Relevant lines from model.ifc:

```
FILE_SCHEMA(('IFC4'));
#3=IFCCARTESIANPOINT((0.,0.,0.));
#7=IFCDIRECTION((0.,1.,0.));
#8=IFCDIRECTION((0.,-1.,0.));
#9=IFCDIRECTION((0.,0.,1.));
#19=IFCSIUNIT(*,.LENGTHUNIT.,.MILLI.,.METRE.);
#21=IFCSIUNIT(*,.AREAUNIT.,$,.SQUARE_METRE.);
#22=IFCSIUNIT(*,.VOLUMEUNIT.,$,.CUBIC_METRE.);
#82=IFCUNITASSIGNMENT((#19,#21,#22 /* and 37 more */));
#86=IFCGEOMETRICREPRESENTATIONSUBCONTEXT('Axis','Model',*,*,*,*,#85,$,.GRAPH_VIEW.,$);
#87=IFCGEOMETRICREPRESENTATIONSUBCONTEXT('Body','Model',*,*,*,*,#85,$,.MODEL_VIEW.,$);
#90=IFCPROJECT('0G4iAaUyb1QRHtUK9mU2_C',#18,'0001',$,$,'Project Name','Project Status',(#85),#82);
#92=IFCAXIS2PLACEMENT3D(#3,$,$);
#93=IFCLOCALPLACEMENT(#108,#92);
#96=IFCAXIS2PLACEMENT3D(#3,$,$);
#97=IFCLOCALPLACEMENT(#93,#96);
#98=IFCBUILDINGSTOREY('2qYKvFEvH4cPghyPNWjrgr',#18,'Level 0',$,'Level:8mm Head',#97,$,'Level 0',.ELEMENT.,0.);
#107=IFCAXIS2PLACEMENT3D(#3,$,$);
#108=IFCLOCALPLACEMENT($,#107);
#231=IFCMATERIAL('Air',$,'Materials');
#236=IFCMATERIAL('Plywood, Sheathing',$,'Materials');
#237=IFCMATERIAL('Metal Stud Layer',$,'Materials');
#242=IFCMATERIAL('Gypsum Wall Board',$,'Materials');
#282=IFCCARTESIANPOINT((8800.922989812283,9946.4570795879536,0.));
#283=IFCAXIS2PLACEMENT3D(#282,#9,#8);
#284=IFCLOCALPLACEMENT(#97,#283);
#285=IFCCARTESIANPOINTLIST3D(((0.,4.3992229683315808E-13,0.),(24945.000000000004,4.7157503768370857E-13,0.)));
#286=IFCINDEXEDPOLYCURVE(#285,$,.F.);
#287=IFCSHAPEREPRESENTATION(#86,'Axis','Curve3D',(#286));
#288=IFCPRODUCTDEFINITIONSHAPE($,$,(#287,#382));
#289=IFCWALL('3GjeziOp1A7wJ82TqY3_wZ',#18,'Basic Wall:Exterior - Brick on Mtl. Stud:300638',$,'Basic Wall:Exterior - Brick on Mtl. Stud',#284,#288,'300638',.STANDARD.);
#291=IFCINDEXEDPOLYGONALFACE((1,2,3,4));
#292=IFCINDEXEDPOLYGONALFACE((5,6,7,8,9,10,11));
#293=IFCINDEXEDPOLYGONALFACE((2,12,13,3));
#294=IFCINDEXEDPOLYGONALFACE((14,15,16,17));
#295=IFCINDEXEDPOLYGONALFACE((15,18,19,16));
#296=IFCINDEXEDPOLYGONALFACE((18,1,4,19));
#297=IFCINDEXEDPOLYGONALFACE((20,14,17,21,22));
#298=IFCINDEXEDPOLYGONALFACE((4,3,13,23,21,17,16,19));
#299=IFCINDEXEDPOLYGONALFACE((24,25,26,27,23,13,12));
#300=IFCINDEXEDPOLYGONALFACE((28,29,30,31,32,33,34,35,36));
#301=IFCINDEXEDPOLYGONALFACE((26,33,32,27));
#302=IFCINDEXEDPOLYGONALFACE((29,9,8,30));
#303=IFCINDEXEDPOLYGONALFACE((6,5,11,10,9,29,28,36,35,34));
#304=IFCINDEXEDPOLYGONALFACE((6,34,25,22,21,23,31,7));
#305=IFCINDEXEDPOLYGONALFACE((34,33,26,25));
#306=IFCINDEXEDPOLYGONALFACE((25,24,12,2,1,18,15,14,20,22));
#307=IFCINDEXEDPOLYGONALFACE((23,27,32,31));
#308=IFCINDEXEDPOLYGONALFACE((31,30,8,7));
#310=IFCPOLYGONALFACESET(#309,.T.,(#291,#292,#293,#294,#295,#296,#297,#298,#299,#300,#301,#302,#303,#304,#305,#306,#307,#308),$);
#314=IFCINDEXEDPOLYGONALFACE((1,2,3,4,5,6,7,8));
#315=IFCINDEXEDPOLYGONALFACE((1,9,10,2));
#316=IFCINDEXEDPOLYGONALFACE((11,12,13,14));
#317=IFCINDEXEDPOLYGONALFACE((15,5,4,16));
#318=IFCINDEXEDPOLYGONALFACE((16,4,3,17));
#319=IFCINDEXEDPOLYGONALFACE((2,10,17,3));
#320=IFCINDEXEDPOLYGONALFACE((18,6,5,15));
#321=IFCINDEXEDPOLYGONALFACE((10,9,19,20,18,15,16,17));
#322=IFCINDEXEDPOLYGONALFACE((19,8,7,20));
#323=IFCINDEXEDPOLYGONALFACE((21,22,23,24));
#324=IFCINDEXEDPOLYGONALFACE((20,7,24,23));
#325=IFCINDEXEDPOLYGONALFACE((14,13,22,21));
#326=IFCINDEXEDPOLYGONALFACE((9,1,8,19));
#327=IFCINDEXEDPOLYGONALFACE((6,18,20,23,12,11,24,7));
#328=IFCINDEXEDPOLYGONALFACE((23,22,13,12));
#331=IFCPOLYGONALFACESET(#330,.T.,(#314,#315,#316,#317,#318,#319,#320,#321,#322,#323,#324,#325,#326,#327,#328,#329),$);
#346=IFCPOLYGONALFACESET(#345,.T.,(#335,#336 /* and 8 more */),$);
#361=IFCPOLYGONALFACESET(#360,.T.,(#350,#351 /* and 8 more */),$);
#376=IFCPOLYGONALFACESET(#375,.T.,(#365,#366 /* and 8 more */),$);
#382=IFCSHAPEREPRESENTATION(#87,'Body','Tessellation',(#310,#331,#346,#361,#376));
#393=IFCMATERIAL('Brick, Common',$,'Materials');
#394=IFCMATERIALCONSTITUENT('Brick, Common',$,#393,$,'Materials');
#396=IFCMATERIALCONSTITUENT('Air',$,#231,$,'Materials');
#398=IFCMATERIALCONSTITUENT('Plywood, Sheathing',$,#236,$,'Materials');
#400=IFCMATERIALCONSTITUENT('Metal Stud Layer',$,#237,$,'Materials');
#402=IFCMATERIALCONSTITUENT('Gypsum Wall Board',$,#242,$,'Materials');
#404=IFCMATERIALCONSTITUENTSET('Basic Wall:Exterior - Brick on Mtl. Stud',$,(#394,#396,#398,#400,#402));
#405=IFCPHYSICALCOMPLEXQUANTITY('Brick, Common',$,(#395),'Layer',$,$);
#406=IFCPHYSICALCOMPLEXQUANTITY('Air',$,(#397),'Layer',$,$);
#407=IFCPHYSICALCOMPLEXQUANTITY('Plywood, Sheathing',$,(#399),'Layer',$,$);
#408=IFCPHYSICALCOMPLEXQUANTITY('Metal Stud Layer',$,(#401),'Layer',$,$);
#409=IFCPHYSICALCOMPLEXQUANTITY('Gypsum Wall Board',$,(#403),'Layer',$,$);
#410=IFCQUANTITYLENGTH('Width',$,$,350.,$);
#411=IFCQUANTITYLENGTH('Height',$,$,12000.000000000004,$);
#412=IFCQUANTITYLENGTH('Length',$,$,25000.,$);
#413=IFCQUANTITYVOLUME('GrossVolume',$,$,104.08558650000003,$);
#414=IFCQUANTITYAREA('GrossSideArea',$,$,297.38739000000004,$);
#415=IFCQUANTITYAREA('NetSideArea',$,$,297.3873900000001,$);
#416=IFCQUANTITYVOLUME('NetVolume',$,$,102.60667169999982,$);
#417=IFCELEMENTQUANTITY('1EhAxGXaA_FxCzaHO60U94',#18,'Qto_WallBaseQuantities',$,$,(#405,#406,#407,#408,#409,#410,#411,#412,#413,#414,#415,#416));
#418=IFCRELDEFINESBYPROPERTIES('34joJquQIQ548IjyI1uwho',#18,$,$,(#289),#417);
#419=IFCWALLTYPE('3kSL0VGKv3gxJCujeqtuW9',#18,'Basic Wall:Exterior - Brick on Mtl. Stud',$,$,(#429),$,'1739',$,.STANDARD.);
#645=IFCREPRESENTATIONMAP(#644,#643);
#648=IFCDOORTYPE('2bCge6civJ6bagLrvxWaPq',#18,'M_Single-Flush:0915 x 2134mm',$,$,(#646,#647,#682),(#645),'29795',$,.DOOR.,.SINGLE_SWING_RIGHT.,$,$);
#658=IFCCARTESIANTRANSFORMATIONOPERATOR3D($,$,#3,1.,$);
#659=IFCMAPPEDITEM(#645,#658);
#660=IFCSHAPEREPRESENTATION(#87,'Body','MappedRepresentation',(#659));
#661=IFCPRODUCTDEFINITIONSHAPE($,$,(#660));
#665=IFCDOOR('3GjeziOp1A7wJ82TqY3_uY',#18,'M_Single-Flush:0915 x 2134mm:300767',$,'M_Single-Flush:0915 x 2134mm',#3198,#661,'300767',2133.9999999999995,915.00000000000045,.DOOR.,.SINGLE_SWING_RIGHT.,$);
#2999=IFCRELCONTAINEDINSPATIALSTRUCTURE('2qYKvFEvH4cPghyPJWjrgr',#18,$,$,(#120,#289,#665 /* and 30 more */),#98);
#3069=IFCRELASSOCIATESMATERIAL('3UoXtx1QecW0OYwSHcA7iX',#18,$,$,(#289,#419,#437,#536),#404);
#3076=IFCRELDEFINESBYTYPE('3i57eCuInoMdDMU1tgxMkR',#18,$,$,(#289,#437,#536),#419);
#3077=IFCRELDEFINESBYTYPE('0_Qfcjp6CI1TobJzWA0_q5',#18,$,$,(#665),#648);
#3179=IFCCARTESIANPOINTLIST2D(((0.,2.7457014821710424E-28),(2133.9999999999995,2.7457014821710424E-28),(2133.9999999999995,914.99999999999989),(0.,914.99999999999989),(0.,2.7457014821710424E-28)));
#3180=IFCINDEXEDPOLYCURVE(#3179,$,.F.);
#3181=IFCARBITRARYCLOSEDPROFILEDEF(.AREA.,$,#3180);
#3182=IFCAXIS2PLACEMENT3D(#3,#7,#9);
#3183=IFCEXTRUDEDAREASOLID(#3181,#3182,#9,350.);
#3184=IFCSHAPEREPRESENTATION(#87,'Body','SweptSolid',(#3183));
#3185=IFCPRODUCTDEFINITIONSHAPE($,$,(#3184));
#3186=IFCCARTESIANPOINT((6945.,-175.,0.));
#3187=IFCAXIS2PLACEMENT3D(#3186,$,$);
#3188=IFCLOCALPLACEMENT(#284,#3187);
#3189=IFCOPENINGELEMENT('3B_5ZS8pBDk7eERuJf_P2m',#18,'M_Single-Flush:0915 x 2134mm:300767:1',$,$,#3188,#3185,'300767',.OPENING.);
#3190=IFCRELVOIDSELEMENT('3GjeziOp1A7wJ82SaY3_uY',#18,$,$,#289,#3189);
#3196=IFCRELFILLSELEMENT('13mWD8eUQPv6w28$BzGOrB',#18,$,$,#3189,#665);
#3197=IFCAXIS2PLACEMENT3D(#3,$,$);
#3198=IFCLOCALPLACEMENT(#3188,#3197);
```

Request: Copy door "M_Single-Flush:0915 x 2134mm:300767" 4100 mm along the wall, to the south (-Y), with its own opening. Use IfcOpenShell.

```python
import ifcopenshell
import ifcopenshell.api.feature
import ifcopenshell.api.geometry
import ifcopenshell.api.pset
import ifcopenshell.api.root
import ifcopenshell.geom
import ifcopenshell.util.element
import ifcopenshell.util.placement
import ifcopenshell.util.shape
import ifcopenshell.util.unit

model = ifcopenshell.open("model.ifc")
area_scale = ifcopenshell.util.unit.calculate_unit_scale(model, "AREAUNIT")
volume_scale = ifcopenshell.util.unit.calculate_unit_scale(model, "VOLUMEUNIT")
settings = ifcopenshell.geom.settings()


def volume(element):
    """Net volume in cubic metres, openings subtracted."""
    shape = ifcopenshell.geom.create_shape(settings, element)
    return ifcopenshell.util.shape.get_volume(shape.geometry)


def reuse_history(source, copy):
    """copy_class also copies each property set's owner history, people and application; keep the originals."""
    for rel in copy.IsDefinedBy:
        if rel.is_a("IfcRelDefinesByProperties") and (history := rel.RelatingPropertyDefinition.OwnerHistory):
            rel.RelatingPropertyDefinition.OwnerHistory = source.OwnerHistory
            ifcopenshell.util.element.remove_deep2(model, history)


door = model.by_id(665)
opening = door.FillsVoids[0].RelatingOpeningElement
wall = opening.VoidsElements[0].RelatingBuildingElement
before = volume(wall)
shift = ifcopenshell.util.placement.get_local_placement(wall.ObjectPlacement)[:3, 0] * 4100.0

# copy_class copies the void relationship, type, container and properties, but no geometry.
new_opening = ifcopenshell.api.root.copy_class(model, product=opening)
new_opening.Representation = ifcopenshell.util.element.copy_deep(
    model, opening.Representation, exclude=["IfcGeometricRepresentationContext", "IfcRepresentationMap"]
)
new_opening.Name = "M_Single-Flush:0915 x 2134mm"
new_opening.Tag = None
reuse_history(opening, new_opening)
new_door = ifcopenshell.api.root.copy_class(model, product=door)
new_door.Representation = ifcopenshell.util.element.copy_deep(
    model, door.Representation, exclude=["IfcGeometricRepresentationContext", "IfcRepresentationMap"]
)
new_door.Name = "M_Single-Flush:0915 x 2134mm"
new_door.Tag = None
reuse_history(door, new_door)
ifcopenshell.api.feature.add_filling(model, opening=new_opening, element=new_door)

for old, new in ((opening, new_opening), (door, new_door)):
    matrix = ifcopenshell.util.placement.get_local_placement(old.ObjectPlacement)
    matrix[:3, 3] += shift
    ifcopenshell.api.geometry.edit_object_placement(model, product=new, matrix=matrix, is_si=False)

after = volume(wall)
thickness = 0.35  # wall thickness in metres

# Update the wall's stored quantities.
qto = model.by_id(ifcopenshell.util.element.get_pset(wall, "Qto_WallBaseQuantities", should_inherit=False)["id"])
ifcopenshell.api.pset.edit_qto(model, qto=qto, properties={
    "NetSideArea": after / thickness / area_scale,
    "NetVolume": after / volume_scale,
})

print(f"wall volume {before:.3f} -> {after:.3f} m3")

model.write("model_updated.ifc")
```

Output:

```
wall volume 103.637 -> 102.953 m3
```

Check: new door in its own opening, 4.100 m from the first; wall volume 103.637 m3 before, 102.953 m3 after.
